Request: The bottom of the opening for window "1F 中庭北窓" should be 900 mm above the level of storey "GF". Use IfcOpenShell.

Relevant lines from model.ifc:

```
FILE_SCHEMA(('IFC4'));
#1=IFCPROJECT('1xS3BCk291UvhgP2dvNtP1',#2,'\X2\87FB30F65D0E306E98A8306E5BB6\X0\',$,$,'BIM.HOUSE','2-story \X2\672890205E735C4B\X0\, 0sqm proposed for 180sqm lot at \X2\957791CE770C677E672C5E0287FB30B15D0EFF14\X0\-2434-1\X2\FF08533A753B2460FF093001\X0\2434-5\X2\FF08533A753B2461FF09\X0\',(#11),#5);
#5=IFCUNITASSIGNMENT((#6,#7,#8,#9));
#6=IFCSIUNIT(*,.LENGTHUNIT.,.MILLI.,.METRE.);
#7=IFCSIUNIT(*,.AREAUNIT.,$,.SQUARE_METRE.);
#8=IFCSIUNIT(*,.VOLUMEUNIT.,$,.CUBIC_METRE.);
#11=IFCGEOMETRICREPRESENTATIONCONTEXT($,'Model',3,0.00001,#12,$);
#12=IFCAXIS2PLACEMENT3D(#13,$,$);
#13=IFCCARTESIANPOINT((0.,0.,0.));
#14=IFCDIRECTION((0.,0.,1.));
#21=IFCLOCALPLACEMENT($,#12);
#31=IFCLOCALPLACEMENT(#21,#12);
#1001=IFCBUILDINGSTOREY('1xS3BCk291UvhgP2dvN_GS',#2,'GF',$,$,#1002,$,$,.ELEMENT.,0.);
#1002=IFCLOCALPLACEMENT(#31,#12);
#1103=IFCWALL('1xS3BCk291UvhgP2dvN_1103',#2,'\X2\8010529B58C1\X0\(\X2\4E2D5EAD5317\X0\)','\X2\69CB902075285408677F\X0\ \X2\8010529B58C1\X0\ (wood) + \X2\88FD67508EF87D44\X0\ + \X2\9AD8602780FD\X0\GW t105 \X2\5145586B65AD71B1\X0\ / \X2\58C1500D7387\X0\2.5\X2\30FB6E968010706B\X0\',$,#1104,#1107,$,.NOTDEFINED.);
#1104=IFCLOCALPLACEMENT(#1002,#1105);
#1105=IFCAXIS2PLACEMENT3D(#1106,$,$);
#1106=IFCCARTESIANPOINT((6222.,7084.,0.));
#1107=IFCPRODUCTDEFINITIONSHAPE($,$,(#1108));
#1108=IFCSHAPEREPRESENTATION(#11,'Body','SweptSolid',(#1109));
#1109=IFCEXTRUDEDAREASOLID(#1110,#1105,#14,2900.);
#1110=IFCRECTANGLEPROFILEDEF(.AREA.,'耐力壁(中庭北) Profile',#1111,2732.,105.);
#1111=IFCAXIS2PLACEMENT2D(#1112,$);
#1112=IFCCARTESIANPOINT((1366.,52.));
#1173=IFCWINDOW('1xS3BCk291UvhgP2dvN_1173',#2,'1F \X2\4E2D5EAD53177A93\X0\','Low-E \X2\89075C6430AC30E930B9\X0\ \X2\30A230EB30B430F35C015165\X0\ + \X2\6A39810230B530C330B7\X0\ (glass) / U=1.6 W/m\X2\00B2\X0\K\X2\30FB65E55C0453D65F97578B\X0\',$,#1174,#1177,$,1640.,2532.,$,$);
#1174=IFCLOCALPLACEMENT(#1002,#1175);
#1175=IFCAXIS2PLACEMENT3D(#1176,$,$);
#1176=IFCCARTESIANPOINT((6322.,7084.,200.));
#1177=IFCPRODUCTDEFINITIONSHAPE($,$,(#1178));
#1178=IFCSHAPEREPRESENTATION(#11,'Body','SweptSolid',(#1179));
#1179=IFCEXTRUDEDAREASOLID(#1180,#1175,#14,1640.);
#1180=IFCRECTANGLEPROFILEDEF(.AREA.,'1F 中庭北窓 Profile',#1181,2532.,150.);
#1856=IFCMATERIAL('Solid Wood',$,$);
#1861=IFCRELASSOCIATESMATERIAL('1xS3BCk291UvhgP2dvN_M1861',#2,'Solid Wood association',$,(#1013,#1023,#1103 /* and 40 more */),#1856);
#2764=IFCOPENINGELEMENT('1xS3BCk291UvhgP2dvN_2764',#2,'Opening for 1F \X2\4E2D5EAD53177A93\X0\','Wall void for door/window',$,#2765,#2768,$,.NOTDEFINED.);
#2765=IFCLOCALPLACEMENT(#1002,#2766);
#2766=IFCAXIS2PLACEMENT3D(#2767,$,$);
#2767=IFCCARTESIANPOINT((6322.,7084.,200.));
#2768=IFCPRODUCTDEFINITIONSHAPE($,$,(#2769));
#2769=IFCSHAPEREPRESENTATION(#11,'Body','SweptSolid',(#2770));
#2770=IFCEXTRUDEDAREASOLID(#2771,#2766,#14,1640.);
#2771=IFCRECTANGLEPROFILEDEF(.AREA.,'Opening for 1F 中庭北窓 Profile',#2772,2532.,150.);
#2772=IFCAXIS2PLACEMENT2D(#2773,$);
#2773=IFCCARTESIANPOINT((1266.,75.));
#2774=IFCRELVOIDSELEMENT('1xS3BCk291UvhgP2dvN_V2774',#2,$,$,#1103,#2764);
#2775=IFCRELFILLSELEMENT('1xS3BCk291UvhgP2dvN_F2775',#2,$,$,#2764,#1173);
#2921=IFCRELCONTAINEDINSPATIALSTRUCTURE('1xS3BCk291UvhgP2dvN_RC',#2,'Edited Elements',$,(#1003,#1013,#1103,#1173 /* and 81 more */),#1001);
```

```python
import numpy as np
import ifcopenshell
import ifcopenshell.api.geometry
import ifcopenshell.geom
import ifcopenshell.util.element
import ifcopenshell.util.placement
import ifcopenshell.util.shape
import ifcopenshell.util.unit

model = ifcopenshell.open("model.ifc")
unit_scale = ifcopenshell.util.unit.calculate_unit_scale(model)

window = model.by_guid("1xS3BCk291UvhgP2dvN_1173")
opening = window.FillsVoids[0].RelatingOpeningElement
storey = ifcopenshell.util.element.get_container(window, ifc_class="IfcBuildingStorey")
level = ifcopenshell.util.placement.get_local_placement(storey.ObjectPlacement)[2, 3]

# The opening's origin need not be at the sill, so measure its lowest point.
shape = ifcopenshell.geom.create_shape(ifcopenshell.geom.settings(), opening)
bottom = ifcopenshell.util.shape.get_shape_bottom_elevation(shape, shape.geometry) / unit_scale
dz = level + 0.9 / unit_scale - bottom

shift = np.array([0.0, 0.0, dz])
# The window is not placed relative to its opening, so move both.
for product in (opening, window):
    matrix = ifcopenshell.util.placement.get_local_placement(product.ObjectPlacement)
    matrix[:3, 3] += shift
    ifcopenshell.api.geometry.edit_object_placement(model, product=product, matrix=matrix, is_si=False)

print(f"moved by {dz * unit_scale:+.3f} m")

model.write("model_rev.ifc")
```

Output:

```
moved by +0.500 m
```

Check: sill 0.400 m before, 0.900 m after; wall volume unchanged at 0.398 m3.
